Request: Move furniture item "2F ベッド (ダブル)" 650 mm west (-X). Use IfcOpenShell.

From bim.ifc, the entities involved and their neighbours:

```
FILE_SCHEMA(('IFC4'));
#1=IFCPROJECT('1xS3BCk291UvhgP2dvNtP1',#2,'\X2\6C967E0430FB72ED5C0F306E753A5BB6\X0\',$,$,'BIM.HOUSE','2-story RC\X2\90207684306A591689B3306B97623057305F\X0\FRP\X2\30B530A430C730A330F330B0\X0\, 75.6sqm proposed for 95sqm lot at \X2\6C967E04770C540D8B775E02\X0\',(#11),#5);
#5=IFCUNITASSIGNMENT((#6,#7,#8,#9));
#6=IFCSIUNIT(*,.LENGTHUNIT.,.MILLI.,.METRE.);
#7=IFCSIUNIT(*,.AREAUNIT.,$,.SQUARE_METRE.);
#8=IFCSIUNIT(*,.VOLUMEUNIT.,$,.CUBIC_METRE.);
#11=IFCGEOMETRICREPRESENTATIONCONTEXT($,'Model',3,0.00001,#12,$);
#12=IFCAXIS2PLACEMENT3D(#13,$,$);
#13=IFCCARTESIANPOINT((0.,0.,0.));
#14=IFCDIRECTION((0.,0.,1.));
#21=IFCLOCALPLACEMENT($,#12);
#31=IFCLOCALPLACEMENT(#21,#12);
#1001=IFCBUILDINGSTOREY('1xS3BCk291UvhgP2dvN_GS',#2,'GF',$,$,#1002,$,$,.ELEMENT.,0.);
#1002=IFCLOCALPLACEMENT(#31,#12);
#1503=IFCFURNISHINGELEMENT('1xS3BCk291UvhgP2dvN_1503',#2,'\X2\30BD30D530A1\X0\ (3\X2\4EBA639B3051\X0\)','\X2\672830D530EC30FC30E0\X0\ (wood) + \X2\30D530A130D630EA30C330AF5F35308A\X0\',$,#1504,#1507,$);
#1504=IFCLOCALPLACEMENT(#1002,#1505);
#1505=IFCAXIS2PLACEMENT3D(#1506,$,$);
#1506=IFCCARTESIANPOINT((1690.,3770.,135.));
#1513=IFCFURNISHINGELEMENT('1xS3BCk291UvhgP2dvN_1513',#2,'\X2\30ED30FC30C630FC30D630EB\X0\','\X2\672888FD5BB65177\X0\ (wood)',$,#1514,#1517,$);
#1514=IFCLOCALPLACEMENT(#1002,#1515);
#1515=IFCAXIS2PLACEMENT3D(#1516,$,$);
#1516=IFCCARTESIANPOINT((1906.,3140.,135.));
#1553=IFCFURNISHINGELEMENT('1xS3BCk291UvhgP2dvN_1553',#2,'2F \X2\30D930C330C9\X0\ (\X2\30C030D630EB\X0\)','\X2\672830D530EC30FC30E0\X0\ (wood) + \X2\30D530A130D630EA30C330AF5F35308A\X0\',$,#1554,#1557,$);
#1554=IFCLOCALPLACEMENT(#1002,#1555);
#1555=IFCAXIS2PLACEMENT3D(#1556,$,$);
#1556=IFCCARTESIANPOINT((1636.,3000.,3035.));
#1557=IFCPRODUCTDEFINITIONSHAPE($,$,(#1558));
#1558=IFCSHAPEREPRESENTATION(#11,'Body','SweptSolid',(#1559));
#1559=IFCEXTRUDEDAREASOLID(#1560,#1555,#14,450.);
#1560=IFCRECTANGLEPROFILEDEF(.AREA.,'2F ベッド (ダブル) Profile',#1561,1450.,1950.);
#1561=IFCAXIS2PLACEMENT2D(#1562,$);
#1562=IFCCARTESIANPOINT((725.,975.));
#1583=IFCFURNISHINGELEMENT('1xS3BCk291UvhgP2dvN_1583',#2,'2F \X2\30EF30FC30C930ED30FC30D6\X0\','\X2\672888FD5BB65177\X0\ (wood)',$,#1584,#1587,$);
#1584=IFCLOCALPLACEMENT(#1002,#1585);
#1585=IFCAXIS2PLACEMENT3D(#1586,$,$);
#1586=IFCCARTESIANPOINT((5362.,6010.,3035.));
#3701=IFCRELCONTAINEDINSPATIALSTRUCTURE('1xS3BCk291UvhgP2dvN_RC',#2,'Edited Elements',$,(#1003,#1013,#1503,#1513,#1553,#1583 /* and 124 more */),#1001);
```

```python
import ifcopenshell
import ifcopenshell.api.geometry
import ifcopenshell.util.placement
import ifcopenshell.util.unit

model = ifcopenshell.open("bim.ifc")
unit_scale = ifcopenshell.util.unit.calculate_unit_scale(model)

item = model.by_guid("1xS3BCk291UvhgP2dvN_1553")
matrix = ifcopenshell.util.placement.get_local_placement(item.ObjectPlacement)
matrix[0, 3] -= 0.65 / unit_scale
ifcopenshell.api.geometry.edit_object_placement(model, product=item, matrix=matrix, is_si=False)

print(ifcopenshell.util.placement.get_local_placement(item.ObjectPlacement).round(3) + 0.0)

model.write("bim-out.ifc")
```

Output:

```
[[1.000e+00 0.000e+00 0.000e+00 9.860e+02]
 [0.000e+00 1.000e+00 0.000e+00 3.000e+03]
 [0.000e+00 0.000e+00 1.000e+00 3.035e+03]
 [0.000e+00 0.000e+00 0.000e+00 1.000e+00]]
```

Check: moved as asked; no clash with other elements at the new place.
